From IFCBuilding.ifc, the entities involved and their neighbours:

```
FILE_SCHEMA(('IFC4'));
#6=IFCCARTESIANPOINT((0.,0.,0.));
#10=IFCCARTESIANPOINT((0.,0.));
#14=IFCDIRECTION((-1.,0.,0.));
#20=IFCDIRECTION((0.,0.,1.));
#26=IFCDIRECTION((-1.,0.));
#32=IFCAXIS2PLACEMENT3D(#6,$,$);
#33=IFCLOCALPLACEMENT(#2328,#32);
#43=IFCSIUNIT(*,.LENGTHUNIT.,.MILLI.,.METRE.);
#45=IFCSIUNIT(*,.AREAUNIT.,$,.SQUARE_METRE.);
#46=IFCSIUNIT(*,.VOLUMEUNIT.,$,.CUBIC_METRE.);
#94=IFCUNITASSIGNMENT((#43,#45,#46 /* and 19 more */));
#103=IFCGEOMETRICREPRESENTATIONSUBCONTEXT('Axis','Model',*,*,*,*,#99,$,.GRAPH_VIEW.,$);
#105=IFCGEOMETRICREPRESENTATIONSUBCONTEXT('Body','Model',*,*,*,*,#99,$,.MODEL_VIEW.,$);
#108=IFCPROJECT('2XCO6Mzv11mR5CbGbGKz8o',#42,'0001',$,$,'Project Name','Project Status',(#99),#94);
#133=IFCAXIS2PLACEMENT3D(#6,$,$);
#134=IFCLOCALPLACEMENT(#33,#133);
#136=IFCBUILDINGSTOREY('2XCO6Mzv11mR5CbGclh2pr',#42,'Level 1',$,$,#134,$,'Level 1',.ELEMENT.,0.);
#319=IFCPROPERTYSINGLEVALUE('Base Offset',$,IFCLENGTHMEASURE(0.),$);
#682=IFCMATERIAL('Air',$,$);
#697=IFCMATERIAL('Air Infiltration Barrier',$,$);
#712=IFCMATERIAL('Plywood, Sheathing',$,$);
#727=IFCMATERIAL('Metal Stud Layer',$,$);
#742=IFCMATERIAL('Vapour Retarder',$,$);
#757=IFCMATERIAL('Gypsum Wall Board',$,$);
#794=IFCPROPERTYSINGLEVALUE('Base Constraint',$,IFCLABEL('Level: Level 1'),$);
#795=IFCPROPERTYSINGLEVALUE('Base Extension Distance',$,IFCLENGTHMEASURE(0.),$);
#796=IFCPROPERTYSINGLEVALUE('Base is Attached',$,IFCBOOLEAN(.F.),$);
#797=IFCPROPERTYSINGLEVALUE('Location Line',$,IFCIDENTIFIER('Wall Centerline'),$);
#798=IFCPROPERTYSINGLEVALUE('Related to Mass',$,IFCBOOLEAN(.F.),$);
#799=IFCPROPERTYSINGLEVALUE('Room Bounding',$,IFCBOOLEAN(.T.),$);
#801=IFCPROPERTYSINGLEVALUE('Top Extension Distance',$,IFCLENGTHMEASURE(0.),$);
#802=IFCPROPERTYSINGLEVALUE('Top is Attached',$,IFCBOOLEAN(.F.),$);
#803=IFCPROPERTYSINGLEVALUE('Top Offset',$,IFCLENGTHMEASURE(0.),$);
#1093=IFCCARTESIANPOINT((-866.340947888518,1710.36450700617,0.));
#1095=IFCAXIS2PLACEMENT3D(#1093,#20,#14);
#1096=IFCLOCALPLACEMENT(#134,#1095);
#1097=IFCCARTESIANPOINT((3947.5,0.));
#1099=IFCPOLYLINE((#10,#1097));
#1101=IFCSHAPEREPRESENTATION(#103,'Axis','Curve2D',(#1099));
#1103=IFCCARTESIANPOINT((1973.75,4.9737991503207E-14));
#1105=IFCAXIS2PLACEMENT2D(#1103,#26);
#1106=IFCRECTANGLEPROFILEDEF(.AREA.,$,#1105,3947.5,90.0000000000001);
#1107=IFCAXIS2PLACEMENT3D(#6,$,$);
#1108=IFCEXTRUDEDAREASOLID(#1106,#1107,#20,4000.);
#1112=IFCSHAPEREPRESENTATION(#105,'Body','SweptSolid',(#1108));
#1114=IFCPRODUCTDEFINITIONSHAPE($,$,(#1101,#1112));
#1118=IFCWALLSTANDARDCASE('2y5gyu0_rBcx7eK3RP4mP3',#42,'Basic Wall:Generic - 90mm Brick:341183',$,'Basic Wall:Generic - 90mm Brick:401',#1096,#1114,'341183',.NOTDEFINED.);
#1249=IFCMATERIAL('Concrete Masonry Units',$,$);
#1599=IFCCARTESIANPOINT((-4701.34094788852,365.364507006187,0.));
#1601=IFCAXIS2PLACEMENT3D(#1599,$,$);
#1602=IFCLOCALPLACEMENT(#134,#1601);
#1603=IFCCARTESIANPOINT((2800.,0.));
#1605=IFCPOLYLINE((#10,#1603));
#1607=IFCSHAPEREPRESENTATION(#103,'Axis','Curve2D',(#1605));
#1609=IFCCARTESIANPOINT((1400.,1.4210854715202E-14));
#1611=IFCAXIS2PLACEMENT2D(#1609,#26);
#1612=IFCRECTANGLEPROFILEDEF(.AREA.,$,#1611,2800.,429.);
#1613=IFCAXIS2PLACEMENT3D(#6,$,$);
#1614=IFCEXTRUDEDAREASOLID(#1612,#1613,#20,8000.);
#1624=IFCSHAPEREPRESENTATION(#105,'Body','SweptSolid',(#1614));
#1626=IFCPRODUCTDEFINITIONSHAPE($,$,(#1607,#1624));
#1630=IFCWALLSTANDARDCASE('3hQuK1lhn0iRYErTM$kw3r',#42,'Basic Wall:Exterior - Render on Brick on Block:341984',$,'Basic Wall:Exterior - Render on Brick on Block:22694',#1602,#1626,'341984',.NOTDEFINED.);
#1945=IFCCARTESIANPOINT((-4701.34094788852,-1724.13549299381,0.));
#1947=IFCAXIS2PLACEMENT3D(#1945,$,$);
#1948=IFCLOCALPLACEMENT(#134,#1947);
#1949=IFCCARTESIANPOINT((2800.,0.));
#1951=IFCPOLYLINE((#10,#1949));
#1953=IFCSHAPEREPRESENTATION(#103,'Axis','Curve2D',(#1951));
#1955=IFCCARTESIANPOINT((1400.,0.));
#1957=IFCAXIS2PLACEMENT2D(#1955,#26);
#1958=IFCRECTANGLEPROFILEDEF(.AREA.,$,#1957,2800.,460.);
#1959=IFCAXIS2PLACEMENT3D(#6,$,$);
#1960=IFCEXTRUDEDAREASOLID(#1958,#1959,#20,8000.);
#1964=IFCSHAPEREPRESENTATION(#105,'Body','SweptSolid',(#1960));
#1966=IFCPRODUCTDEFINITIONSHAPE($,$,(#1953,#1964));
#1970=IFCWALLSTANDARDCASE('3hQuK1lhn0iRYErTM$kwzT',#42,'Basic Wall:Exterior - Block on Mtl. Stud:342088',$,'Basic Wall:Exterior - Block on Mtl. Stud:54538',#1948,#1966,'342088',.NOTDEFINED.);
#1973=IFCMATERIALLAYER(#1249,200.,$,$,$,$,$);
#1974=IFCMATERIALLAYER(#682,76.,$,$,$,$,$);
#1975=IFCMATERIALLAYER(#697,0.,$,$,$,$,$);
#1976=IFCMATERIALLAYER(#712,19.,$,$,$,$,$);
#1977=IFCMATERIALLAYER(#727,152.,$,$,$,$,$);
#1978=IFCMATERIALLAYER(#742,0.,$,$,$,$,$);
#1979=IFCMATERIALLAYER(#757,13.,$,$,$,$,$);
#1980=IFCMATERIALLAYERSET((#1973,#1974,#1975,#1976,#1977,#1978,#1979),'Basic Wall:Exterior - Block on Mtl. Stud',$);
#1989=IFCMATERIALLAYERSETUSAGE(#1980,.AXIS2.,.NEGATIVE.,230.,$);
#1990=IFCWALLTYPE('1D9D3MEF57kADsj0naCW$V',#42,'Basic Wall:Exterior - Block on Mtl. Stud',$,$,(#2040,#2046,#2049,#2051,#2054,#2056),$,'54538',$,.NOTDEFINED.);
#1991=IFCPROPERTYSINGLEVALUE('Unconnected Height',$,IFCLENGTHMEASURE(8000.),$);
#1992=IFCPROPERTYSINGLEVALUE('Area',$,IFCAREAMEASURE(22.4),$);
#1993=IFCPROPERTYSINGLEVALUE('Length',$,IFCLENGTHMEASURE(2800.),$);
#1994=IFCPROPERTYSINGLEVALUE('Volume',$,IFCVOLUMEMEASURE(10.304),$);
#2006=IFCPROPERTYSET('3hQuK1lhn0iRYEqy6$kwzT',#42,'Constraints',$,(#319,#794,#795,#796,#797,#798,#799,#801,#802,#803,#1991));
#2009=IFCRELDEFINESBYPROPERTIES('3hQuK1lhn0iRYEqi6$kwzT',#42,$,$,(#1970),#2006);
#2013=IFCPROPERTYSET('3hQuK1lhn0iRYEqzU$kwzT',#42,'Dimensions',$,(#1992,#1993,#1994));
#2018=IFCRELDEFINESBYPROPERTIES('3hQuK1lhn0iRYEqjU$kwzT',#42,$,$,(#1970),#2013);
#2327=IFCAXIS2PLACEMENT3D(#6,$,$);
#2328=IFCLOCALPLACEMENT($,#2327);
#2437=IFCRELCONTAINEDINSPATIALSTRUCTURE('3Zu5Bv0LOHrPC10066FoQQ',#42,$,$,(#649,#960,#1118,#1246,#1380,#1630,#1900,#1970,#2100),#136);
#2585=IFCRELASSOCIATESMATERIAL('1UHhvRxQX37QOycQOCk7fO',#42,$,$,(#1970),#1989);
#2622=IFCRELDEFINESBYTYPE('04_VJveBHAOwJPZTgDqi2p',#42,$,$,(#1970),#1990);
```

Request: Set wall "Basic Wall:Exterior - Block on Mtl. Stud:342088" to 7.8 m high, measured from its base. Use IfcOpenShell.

```python
import ifcopenshell
import ifcopenshell.api.pset
import ifcopenshell.geom
import ifcopenshell.util.element
import ifcopenshell.util.representation
import ifcopenshell.util.shape
import ifcopenshell.util.unit

model = ifcopenshell.open("IFCBuilding.ifc")
unit_scale = ifcopenshell.util.unit.calculate_unit_scale(model)
area_scale = ifcopenshell.util.unit.calculate_unit_scale(model, "AREAUNIT")
volume_scale = ifcopenshell.util.unit.calculate_unit_scale(model, "VOLUMEUNIT")
settings = ifcopenshell.geom.settings()


def volume(element):
    """Net volume in cubic metres, openings subtracted."""
    shape = ifcopenshell.geom.create_shape(settings, element)
    return ifcopenshell.util.shape.get_volume(shape.geometry)


wall = model.by_id(1970)
before = volume(wall)

body = ifcopenshell.util.representation.get_representation(wall, "Model", "Body")
solid = body.Items[0]
old_height = solid.Depth
solid.Depth = 7.8 / unit_scale
after = volume(wall)
thickness = 0.46  # wall thickness in metres

# Update the stored height, areas and volumes.
pset = model.by_id(ifcopenshell.util.element.get_pset(wall, "Constraints", should_inherit=False)["id"])
ifcopenshell.api.pset.edit_pset(model, pset=pset, properties={
    "Unconnected Height": model.create_entity("IfcLengthMeasure", solid.Depth),
})
pset = model.by_id(ifcopenshell.util.element.get_pset(wall, "Dimensions", should_inherit=False)["id"])
ifcopenshell.api.pset.edit_pset(model, pset=pset, properties={
    "Area": model.create_entity("IfcAreaMeasure", after / thickness / area_scale),
    "Volume": model.create_entity("IfcVolumeMeasure", after / volume_scale),
})

print(f"height {old_height:g} -> {solid.Depth:g}, volume {before:.3f} -> {after:.3f} m3")

model.write("IFCBuilding_rev.ifc")
```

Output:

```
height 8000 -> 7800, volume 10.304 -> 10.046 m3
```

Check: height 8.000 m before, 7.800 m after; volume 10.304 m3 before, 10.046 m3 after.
